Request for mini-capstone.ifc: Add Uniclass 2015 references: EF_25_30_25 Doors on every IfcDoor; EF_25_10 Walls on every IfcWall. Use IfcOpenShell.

First a look at what the model holds.

```python
import ifcopenshell

model = ifcopenshell.open("mini-capstone.ifc")
print(model.schema)
print("classifications:", [c.Name for c in model.by_type("IfcClassification")])
for ifc_class in ("IfcDoor", "IfcRoof", "IfcStair", "IfcWall", "IfcWindow"):
    print(ifc_class, len(model.by_type(ifc_class)))
```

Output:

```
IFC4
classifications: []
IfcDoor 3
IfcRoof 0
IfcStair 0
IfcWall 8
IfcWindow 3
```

```python
import ifcopenshell
import ifcopenshell.api.classification

model = ifcopenshell.open("mini-capstone.ifc")

system = ifcopenshell.api.classification.add_classification(model, classification="Uniclass 2015")

codes = {
    "IfcDoor": ("EF_25_30_25", "Doors"),
    "IfcWall": ("EF_25_10", "Walls"),
}
for ifc_class, (code, name) in codes.items():
    products = model.by_type(ifc_class)
    ifcopenshell.api.classification.add_reference(
        model, products=products, classification=system, identification=code, name=name
    )
    print(code, len(products))

model.write("mini-capstone_rev.ifc")
```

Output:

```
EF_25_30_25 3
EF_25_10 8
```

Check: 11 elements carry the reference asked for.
